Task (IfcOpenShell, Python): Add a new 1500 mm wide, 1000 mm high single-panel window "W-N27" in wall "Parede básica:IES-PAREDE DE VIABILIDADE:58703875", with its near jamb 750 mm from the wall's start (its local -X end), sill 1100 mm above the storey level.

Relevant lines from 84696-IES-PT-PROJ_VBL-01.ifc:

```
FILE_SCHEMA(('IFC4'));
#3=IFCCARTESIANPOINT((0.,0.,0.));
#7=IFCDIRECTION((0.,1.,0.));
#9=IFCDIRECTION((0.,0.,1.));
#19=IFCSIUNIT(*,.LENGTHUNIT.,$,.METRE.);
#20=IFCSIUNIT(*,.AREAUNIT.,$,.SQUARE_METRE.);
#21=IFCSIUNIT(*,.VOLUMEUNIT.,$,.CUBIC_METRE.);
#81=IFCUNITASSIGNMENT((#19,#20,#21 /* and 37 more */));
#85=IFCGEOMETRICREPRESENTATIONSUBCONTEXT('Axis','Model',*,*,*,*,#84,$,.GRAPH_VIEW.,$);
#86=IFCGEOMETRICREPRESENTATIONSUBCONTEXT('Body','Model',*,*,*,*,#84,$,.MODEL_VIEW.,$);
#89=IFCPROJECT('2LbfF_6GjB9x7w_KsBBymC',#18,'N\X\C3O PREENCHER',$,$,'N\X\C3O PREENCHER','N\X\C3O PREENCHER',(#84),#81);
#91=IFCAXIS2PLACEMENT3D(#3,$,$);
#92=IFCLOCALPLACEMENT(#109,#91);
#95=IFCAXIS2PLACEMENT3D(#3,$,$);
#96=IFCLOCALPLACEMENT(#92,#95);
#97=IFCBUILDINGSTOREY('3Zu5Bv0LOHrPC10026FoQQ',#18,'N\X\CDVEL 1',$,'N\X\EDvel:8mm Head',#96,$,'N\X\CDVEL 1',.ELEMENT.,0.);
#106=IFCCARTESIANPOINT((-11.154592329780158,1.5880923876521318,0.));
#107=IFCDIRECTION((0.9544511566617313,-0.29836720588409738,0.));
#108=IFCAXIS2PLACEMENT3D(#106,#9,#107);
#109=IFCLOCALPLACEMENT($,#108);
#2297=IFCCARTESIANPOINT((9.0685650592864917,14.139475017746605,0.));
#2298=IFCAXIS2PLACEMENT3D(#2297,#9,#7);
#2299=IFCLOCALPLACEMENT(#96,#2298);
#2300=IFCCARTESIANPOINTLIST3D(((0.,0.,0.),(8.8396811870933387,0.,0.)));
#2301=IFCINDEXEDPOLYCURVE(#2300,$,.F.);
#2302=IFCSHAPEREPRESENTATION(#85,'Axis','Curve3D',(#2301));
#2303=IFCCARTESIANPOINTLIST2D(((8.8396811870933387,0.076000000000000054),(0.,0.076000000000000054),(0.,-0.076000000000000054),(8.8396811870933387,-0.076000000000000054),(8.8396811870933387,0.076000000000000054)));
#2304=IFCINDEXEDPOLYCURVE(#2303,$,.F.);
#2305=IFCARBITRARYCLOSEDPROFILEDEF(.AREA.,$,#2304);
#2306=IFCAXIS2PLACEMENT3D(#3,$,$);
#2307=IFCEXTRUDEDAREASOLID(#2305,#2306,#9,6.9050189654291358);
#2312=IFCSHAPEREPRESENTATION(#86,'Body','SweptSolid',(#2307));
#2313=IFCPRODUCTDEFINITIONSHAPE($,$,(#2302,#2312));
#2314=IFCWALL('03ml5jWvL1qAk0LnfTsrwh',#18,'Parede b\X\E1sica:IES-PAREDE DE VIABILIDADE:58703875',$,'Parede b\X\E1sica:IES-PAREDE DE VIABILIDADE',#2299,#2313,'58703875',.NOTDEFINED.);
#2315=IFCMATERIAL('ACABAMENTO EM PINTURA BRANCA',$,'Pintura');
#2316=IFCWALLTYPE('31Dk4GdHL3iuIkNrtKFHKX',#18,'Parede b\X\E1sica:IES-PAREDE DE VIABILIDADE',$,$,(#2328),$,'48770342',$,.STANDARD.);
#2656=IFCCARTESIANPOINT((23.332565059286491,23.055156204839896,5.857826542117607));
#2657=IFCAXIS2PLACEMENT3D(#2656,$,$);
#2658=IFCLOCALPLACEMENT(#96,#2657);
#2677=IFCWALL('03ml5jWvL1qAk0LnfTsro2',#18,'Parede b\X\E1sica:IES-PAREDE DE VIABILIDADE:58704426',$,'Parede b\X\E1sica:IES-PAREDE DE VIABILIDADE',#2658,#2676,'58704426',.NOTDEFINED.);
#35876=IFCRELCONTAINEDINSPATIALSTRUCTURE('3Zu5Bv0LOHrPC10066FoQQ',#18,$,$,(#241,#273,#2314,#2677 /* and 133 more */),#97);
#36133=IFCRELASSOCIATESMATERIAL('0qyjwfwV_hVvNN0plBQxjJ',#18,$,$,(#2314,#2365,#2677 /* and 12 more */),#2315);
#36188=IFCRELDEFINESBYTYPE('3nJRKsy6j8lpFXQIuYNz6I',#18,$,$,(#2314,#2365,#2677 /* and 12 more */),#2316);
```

```python
import numpy as np
import ifcopenshell
import ifcopenshell.api.feature
import ifcopenshell.api.geometry
import ifcopenshell.api.root
import ifcopenshell.api.spatial
import ifcopenshell.geom
import ifcopenshell.util.element
import ifcopenshell.util.placement
import ifcopenshell.util.representation
import ifcopenshell.util.shape
import ifcopenshell.util.unit

model = ifcopenshell.open("84696-IES-PT-PROJ_VBL-01.ifc")
unit_scale = ifcopenshell.util.unit.calculate_unit_scale(model)
settings = ifcopenshell.geom.settings()


def volume(element):
    """Net volume in cubic metres, openings subtracted."""
    shape = ifcopenshell.geom.create_shape(settings, element)
    return ifcopenshell.util.shape.get_volume(shape.geometry)


wall = model.by_guid("03ml5jWvL1qAk0LnfTsrwh")
storey = ifcopenshell.util.element.get_container(wall, ifc_class="IfcBuildingStorey")
context = ifcopenshell.util.representation.get_context(model, "Model", "Body", "MODEL_VIEW")
before = volume(wall)

width, height, from_end, sill = 1.5, 1, 0.75, 1.1  # metres

# The wall runs along its own X axis, and the end named is its -X end.
wall_shape = ifcopenshell.geom.create_shape(settings, wall)
x, y, z = ifcopenshell.util.shape.get_vertices(wall_shape.geometry).T
start = x.min() + from_end
face, thickness = float(y.min()), float(y.max() - y.min())
wall_matrix = ifcopenshell.util.placement.get_local_placement(wall.ObjectPlacement)
level = ifcopenshell.util.placement.get_local_placement(storey.ObjectPlacement)[2, 3]


def in_wall(x, y):
    """Placement at x, y metres in the wall's axes, at sill height."""
    matrix = wall_matrix.copy()
    matrix[:, 3] = wall_matrix @ np.array([x / unit_scale, y / unit_scale, 0.0, 1.0])
    matrix[2, 3] = level + sill / unit_scale
    return matrix


# Opening: a box that overshoots both wall faces by 50 mm.
opening = ifcopenshell.api.root.create_entity(model, ifc_class="IfcOpeningElement", predefined_type="OPENING")
box = ifcopenshell.api.geometry.add_wall_representation(
    model, context=context, length=width, height=height, thickness=thickness + 0.1
)
ifcopenshell.api.geometry.assign_representation(model, product=opening, representation=box)
ifcopenshell.api.geometry.edit_object_placement(model, product=opening, matrix=in_wall(start, face - 0.05), is_si=False)
ifcopenshell.api.feature.add_feature(model, feature=opening, element=wall)

window = ifcopenshell.api.root.create_entity(model, ifc_class="IfcWindow", name="W-N27", predefined_type="WINDOW")
window.OverallWidth, window.OverallHeight = width / unit_scale, height / unit_scale
window.PartitioningType = "SINGLE_PANEL"
body = ifcopenshell.api.geometry.add_window_representation(
    model,
    context=context,
    overall_width=window.OverallWidth,
    overall_height=window.OverallHeight,
    partition_type="SINGLE_PANEL",
)
ifcopenshell.api.geometry.assign_representation(model, product=window, representation=body)
ifcopenshell.api.spatial.assign_container(model, products=[window], relating_structure=storey)
ifcopenshell.api.feature.add_filling(model, opening=opening, element=window)

# Centre the window in the wall's thickness.
ifcopenshell.api.geometry.edit_object_placement(model, product=window, matrix=in_wall(start, face), is_si=False)
window_shape = ifcopenshell.geom.create_shape(settings, window)
depth = ifcopenshell.util.shape.get_vertices(window_shape.geometry)[:, 1]
offset = face + thickness / 2 - (depth.min() + depth.max()) / 2
ifcopenshell.api.geometry.edit_object_placement(model, product=window, matrix=in_wall(start, offset), is_si=False)

after = volume(wall)

print(f"wall volume {before:.3f} -> {after:.3f} m3")

model.write("84696-IES-PT-PROJ_VBL-01_updated.ifc")
```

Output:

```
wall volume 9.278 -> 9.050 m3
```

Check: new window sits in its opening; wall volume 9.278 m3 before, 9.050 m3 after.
